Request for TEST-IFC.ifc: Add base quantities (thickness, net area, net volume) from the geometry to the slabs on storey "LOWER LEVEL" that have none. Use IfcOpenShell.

First a look at what the model holds.

```python
import ifcopenshell
import ifcopenshell.util.element
import ifcopenshell.util.unit

model = ifcopenshell.open("TEST-IFC.ifc")
print(model.schema)
for unit_type in ("LENGTHUNIT", "AREAUNIT", "VOLUMEUNIT"):
    print(unit_type, ifcopenshell.util.unit.calculate_unit_scale(model, unit_type))
storey = next(s for s in model.by_type("IfcBuildingStorey") if s.Name == "LOWER LEVEL")
slabs = [e for e in ifcopenshell.util.element.get_decomposition(storey) if e.is_a("IfcSlab")]
for e in sorted(slabs, key=lambda e: e.id()):
    print(e.id(), e.is_a(), e.Name, list(ifcopenshell.util.element.get_psets(e, qtos_only=True)), sep=" | ")
```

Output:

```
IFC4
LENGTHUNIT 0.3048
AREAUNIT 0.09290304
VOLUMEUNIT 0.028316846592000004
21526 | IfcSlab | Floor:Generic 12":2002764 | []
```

```python
import ifcopenshell
import ifcopenshell.api.pset
import ifcopenshell.geom
import ifcopenshell.util.element
import ifcopenshell.util.shape
import ifcopenshell.util.unit

model = ifcopenshell.open("TEST-IFC.ifc")
unit_scale = ifcopenshell.util.unit.calculate_unit_scale(model)
area_scale = ifcopenshell.util.unit.calculate_unit_scale(model, "AREAUNIT")
volume_scale = ifcopenshell.util.unit.calculate_unit_scale(model, "VOLUMEUNIT")
settings = ifcopenshell.geom.settings()

storey = next(s for s in model.by_type("IfcBuildingStorey") if s.Name == "LOWER LEVEL")
slabs = [e for e in ifcopenshell.util.element.get_decomposition(storey) if e.is_a("IfcSlab")]

for e in sorted(slabs, key=lambda e: e.id()):
    if ifcopenshell.util.element.get_psets(e, qtos_only=True, should_inherit=False):
        continue
    # Geometry comes back in metres, in the element's own axes.
    shape = ifcopenshell.geom.create_shape(settings, e)
    values = {
        "Width": ifcopenshell.util.shape.get_z(shape.geometry) / unit_scale,
        "NetArea": ifcopenshell.util.shape.get_footprint_area(shape.geometry) / area_scale,
        "NetVolume": ifcopenshell.util.shape.get_volume(shape.geometry) / volume_scale,
    }
    qto = ifcopenshell.api.pset.add_qto(model, product=e, name="Qto_SlabBaseQuantities")
    ifcopenshell.api.pset.edit_qto(model, qto=qto, properties=values)
    print(e.id(), {k: round(v, 3) for k, v in values.items()})

model.write("TEST-IFC_rev.ifc")
```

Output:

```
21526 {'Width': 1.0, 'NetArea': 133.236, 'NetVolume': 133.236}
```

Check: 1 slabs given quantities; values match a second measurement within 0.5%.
